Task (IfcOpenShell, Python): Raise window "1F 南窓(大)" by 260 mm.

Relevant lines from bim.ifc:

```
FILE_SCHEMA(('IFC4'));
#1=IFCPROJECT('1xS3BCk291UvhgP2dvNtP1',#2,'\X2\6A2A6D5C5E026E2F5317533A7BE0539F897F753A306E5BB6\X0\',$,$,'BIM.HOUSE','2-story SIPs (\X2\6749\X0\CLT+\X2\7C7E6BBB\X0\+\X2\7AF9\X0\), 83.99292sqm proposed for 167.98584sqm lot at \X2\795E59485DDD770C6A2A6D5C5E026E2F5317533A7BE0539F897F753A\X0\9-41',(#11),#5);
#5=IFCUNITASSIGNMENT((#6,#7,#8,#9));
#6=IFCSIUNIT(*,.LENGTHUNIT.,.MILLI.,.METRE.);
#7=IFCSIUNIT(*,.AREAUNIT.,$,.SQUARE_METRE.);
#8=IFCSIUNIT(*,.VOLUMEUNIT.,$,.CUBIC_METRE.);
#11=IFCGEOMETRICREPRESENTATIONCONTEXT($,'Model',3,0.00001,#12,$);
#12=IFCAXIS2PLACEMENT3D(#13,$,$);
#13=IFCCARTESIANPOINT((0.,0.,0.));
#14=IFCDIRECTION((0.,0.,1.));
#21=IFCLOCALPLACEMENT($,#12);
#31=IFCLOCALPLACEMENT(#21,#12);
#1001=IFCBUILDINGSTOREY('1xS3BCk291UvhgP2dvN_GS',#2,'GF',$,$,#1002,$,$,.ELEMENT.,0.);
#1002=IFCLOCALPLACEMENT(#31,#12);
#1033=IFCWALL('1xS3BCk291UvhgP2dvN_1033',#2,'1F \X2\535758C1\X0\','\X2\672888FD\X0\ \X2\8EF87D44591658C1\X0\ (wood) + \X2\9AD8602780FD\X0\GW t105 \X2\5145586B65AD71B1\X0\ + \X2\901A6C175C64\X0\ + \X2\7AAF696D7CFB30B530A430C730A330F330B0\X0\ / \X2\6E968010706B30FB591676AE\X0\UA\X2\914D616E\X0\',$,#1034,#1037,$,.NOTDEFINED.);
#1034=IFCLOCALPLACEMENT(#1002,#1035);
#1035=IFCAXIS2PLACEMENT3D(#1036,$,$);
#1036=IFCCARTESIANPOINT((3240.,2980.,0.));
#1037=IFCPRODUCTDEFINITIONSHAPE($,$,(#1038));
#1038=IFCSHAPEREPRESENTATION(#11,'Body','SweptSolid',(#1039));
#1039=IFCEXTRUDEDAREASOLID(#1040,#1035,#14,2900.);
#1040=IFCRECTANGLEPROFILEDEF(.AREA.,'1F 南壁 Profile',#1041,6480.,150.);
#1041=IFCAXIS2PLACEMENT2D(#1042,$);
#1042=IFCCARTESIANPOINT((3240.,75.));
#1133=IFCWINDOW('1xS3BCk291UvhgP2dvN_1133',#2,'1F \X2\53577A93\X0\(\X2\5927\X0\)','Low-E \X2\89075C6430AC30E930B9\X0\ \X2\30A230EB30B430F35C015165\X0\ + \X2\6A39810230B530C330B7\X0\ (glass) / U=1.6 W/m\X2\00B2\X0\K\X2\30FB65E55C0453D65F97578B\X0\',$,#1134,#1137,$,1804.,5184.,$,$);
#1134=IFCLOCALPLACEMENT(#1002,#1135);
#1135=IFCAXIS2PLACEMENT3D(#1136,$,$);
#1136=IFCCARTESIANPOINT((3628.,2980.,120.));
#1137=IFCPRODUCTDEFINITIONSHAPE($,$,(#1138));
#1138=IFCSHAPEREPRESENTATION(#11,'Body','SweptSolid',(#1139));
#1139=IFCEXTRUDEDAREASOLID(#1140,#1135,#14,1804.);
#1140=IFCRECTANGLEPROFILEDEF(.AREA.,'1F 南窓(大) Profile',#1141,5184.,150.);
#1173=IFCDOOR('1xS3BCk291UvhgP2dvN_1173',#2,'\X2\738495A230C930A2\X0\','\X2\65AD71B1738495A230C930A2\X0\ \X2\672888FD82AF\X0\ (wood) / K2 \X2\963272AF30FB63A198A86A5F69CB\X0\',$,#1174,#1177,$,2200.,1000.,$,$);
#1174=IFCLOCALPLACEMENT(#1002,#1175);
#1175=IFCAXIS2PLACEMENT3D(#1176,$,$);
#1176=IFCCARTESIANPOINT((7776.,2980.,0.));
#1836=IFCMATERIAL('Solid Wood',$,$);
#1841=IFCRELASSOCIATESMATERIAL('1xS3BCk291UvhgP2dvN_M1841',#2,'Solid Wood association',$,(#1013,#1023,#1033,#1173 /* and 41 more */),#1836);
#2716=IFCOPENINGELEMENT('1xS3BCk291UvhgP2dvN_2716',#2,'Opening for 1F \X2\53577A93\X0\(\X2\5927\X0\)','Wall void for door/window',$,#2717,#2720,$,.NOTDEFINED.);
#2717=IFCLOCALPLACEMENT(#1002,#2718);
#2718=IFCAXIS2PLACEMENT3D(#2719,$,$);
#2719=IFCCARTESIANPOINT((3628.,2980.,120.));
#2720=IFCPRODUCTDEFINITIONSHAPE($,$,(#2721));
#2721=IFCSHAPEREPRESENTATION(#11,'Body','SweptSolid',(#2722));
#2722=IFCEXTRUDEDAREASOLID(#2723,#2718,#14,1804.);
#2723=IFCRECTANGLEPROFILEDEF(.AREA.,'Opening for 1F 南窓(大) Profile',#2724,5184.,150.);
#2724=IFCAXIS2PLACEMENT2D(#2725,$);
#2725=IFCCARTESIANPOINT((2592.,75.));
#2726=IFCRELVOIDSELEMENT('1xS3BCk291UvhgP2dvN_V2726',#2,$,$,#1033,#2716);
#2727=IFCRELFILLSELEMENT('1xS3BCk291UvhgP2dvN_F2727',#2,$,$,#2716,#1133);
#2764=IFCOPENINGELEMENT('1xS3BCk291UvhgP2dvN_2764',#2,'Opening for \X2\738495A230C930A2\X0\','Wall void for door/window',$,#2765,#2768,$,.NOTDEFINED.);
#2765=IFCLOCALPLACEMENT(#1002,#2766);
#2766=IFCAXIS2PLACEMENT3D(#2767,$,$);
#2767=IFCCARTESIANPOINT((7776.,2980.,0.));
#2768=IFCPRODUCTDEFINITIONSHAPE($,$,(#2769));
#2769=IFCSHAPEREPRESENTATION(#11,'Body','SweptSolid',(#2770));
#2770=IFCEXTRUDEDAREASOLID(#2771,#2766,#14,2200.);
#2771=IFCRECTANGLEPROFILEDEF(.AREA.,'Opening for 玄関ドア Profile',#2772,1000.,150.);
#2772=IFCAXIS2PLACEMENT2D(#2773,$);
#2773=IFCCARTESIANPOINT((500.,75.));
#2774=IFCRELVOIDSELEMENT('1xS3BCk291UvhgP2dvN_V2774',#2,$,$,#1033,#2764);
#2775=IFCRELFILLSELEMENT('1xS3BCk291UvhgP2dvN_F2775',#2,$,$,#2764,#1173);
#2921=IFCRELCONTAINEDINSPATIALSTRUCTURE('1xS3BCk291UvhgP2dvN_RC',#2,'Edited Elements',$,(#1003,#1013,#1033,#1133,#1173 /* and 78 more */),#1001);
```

```python
import numpy as np
import ifcopenshell
import ifcopenshell.api.geometry
import ifcopenshell.util.placement
import ifcopenshell.util.unit

model = ifcopenshell.open("bim.ifc")
unit_scale = ifcopenshell.util.unit.calculate_unit_scale(model)

window = model.by_guid("1xS3BCk291UvhgP2dvN_1133")
opening = window.FillsVoids[0].RelatingOpeningElement
dz = 260.0

shift = np.array([0.0, 0.0, dz])
# The window is not placed relative to its opening, so move both.
for product in (opening, window):
    matrix = ifcopenshell.util.placement.get_local_placement(product.ObjectPlacement)
    matrix[:3, 3] += shift
    ifcopenshell.api.geometry.edit_object_placement(model, product=product, matrix=matrix, is_si=False)

print(f"moved by {dz * unit_scale:+.3f} m")

model.write("bim_edited.ifc")
```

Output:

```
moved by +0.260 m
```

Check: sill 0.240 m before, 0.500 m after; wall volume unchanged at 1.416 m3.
